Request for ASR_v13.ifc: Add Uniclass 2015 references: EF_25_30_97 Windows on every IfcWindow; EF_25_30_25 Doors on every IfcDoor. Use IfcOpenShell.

First a look at what the model holds.

```python
import ifcopenshell

model = ifcopenshell.open("ASR_v13.ifc")
print(model.schema)
print("classifications:", [c.Name for c in model.by_type("IfcClassification")])
for ifc_class in ("IfcDoor", "IfcRoof", "IfcStair", "IfcWall", "IfcWindow"):
    print(ifc_class, len(model.by_type(ifc_class)))
```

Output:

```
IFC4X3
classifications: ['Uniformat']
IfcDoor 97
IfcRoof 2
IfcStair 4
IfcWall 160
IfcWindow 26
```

```python
import ifcopenshell
import ifcopenshell.api.classification

model = ifcopenshell.open("ASR_v13.ifc")

system = ifcopenshell.api.classification.add_classification(model, classification="Uniclass 2015")

codes = {
    "IfcWindow": ("EF_25_30_97", "Windows"),
    "IfcDoor": ("EF_25_30_25", "Doors"),
}
for ifc_class, (code, name) in codes.items():
    products = model.by_type(ifc_class)
    ifcopenshell.api.classification.add_reference(
        model, products=products, classification=system, identification=code, name=name
    )
    print(code, len(products))

model.write("ASR_v13_edited.ifc")
```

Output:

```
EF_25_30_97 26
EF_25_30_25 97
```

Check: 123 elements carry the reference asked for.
